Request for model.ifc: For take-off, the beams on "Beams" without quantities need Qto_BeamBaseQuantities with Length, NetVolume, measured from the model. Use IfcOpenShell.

First a look at what the model holds.

```python
import ifcopenshell
import ifcopenshell.util.element
import ifcopenshell.util.unit

model = ifcopenshell.open("model.ifc")
print(model.schema)
for unit_type in ("LENGTHUNIT", "AREAUNIT", "VOLUMEUNIT"):
    print(unit_type, ifcopenshell.util.unit.calculate_unit_scale(model, unit_type))
storey = next(s for s in model.by_type("IfcBuildingStorey") if s.Name == "Beams")
beams = [e for e in ifcopenshell.util.element.get_decomposition(storey) if e.is_a("IfcBeam")]
for e in sorted(beams, key=lambda e: e.id()):
    print(e.id(), e.is_a(), e.Name, list(ifcopenshell.util.element.get_psets(e, qtos_only=True)), sep=" | ")
```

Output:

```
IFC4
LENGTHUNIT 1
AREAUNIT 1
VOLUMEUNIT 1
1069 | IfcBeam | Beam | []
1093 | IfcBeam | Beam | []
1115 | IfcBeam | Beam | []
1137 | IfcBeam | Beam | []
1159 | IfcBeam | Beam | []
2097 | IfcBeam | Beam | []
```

```python
import ifcopenshell
import ifcopenshell.api.pset
import ifcopenshell.geom
import ifcopenshell.util.element
import ifcopenshell.util.shape
import ifcopenshell.util.unit

model = ifcopenshell.open("model.ifc")
unit_scale = ifcopenshell.util.unit.calculate_unit_scale(model)
volume_scale = ifcopenshell.util.unit.calculate_unit_scale(model, "VOLUMEUNIT")
settings = ifcopenshell.geom.settings()

storey = next(s for s in model.by_type("IfcBuildingStorey") if s.Name == "Beams")
beams = [e for e in ifcopenshell.util.element.get_decomposition(storey) if e.is_a("IfcBeam")]

for e in sorted(beams, key=lambda e: e.id()):
    if ifcopenshell.util.element.get_psets(e, qtos_only=True, should_inherit=False):
        continue
    # Geometry comes back in metres, in the element's own axes.
    shape = ifcopenshell.geom.create_shape(settings, e)
    values = {
        "Length": ifcopenshell.util.shape.get_max_xyz(shape.geometry) / unit_scale,
        "NetVolume": ifcopenshell.util.shape.get_volume(shape.geometry) / volume_scale,
    }
    qto = ifcopenshell.api.pset.add_qto(model, product=e, name="Qto_BeamBaseQuantities")
    ifcopenshell.api.pset.edit_qto(model, qto=qto, properties=values)
    print(e.id(), {k: round(v, 3) for k, v in values.items()})

model.write("model_edited.ifc")
```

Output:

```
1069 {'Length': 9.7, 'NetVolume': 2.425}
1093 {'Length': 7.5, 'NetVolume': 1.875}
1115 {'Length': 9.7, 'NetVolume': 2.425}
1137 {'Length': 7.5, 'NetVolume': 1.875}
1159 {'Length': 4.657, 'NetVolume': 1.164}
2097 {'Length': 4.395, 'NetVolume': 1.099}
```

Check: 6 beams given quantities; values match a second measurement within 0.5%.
